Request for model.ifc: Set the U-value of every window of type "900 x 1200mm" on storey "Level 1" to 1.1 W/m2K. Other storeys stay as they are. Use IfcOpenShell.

First a look at what the model holds.

```python
import ifcopenshell
import ifcopenshell.util.element

model = ifcopenshell.open("model.ifc")
print(model.schema)
storey = next(s for s in model.by_type("IfcBuildingStorey") if s.Name == "Level 1")
windows = [e for e in ifcopenshell.util.element.get_decomposition(storey) if e.is_a("IfcWindow")]
seen = {}
for e in windows:
    element_type = ifcopenshell.util.element.get_type(e)
    key = (element_type.Name if element_type != e and element_type else None, ifcopenshell.util.element.get_pset(e, "Pset_WindowCommon", "ThermalTransmittance"))
    seen[key] = seen.get(key, 0) + 1
for (name, value), count in sorted(seen.items(), key=str):
    print(count, "x", name, "|", value)
```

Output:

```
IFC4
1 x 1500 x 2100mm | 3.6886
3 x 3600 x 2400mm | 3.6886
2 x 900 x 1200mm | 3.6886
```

```python
import ifcopenshell
import ifcopenshell.api.pset
import ifcopenshell.util.element

model = ifcopenshell.open("model.ifc")

storey = next(s for s in model.by_type("IfcBuildingStorey") if s.Name == "Level 1")
windows = [e for e in ifcopenshell.util.element.get_decomposition(storey) if e.is_a("IfcWindow")]

count = 0
for e in windows:
    element_type = ifcopenshell.util.element.get_type(e)
    if element_type in (None, e) or element_type.Name != "900 x 1200mm":
        continue
    # add_pset returns the element's existing set when there is one.
    pset = ifcopenshell.api.pset.add_pset(model, product=e, name="Pset_WindowCommon")
    ifcopenshell.api.pset.edit_pset(model, pset=pset, properties={"ThermalTransmittance": 1.1})
    count += 1

print(count, "windows updated")

model.write("model_rev.ifc")
```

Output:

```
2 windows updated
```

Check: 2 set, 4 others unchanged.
